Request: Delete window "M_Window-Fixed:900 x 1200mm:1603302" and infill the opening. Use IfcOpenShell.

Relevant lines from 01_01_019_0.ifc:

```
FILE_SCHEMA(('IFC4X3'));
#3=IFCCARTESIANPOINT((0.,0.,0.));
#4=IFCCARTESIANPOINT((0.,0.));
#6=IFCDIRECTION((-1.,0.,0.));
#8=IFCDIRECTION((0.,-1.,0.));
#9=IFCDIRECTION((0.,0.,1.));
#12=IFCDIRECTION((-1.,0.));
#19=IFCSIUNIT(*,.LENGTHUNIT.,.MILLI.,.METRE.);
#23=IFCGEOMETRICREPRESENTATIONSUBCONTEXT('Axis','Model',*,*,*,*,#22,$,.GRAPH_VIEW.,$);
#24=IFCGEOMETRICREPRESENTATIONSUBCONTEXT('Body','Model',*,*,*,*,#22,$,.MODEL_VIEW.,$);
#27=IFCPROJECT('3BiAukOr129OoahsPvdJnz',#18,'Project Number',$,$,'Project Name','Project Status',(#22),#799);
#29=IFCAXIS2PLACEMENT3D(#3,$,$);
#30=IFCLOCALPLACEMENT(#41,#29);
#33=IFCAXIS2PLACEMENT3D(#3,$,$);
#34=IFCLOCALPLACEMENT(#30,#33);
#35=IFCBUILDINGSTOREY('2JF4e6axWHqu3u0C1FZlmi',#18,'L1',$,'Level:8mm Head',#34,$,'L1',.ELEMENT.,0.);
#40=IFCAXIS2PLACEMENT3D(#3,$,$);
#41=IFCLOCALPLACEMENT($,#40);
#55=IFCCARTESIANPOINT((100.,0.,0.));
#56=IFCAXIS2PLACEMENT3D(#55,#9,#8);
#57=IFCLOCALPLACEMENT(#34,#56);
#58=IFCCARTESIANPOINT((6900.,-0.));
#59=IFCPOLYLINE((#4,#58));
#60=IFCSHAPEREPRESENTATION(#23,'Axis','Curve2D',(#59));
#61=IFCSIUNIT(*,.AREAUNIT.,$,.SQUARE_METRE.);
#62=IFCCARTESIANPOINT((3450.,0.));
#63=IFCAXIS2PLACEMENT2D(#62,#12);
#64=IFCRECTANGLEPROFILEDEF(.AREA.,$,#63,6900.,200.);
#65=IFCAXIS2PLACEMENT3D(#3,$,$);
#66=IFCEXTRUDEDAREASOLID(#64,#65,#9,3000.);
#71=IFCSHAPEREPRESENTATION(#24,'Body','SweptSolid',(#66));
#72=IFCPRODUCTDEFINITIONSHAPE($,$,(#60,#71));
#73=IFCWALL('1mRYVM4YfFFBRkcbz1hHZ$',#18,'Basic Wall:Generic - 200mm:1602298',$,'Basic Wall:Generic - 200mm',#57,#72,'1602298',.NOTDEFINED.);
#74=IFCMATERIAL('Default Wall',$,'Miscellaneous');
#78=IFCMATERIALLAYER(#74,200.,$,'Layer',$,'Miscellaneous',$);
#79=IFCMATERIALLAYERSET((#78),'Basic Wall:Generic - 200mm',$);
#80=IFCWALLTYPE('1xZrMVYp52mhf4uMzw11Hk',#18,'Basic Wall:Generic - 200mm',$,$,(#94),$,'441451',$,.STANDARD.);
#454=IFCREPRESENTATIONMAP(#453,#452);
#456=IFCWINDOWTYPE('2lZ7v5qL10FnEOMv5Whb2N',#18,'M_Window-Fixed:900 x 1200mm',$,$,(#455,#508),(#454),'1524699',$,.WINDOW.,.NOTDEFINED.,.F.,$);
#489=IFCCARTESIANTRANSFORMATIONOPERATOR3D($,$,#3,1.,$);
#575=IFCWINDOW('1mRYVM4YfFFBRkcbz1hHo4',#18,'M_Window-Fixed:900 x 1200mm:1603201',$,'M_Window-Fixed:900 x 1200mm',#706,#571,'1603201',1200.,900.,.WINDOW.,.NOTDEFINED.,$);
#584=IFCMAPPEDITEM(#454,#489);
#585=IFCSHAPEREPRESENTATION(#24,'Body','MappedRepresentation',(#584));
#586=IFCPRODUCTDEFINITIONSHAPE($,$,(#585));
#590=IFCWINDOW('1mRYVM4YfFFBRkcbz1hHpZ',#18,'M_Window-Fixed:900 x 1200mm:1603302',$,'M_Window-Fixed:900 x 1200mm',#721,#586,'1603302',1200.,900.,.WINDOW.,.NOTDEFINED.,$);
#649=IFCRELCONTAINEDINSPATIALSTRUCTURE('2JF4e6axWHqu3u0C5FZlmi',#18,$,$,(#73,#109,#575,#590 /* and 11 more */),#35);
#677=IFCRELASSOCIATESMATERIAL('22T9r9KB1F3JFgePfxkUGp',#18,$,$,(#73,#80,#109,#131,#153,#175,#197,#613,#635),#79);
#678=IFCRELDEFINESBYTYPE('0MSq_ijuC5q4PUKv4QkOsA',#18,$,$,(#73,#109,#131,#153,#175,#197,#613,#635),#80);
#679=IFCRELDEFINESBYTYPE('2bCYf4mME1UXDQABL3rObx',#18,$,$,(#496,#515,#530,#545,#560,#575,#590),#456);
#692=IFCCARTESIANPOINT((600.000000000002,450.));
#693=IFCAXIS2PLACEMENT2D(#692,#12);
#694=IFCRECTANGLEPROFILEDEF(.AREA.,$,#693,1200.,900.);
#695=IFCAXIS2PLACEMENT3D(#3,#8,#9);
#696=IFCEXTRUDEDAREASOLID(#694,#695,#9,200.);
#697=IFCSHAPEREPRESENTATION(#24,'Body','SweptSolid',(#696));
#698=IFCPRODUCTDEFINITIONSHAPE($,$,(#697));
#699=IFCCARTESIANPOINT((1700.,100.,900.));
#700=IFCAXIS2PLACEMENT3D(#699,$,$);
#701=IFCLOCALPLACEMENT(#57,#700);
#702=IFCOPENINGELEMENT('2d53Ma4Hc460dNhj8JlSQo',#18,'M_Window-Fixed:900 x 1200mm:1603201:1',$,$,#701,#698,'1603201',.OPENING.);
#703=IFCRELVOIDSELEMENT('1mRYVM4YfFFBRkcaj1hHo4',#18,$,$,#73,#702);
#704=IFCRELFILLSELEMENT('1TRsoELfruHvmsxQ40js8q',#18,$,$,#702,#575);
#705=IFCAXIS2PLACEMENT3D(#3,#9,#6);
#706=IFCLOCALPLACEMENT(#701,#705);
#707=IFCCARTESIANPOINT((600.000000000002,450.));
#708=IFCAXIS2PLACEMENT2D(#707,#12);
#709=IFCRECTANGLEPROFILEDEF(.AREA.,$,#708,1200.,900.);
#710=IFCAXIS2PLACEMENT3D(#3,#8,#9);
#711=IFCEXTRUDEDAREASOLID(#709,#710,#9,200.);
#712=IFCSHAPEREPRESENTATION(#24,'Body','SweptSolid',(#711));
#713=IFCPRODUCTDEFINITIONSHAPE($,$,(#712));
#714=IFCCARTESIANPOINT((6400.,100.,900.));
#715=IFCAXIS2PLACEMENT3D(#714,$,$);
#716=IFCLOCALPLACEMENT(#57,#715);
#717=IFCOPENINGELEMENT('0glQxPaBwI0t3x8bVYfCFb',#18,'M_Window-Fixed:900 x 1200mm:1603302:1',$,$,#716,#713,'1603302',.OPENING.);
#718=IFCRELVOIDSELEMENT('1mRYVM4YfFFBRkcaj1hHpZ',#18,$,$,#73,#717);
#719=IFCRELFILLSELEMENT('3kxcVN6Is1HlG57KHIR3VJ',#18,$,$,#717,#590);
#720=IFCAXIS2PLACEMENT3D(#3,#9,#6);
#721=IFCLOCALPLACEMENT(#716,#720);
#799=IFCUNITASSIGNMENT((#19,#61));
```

```python
import ifcopenshell
import ifcopenshell.api.feature
import ifcopenshell.api.root
import ifcopenshell.geom
import ifcopenshell.util.shape

model = ifcopenshell.open("01_01_019_0.ifc")
settings = ifcopenshell.geom.settings()


def volume(element):
    """Net volume in cubic metres, openings subtracted."""
    shape = ifcopenshell.geom.create_shape(settings, element)
    return ifcopenshell.util.shape.get_volume(shape.geometry)


window = model.by_guid("1mRYVM4YfFFBRkcbz1hHpZ")
opening = window.FillsVoids[0].RelatingOpeningElement
wall = opening.VoidsElements[0].RelatingBuildingElement
before = volume(wall)

ifcopenshell.api.root.remove_product(model, product=window)
ifcopenshell.api.feature.remove_feature(model, feature=opening)

after = volume(wall)

print(f"wall volume {before:.3f} -> {after:.3f} m3")

model.write("01_01_019_0_updated.ifc")
```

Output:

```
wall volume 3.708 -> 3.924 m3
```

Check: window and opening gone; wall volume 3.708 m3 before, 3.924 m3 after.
